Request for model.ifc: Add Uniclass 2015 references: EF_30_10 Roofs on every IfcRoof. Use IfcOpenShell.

First a look at what the model holds.

```python
import ifcopenshell

model = ifcopenshell.open("model.ifc")
print(model.schema)
print("classifications:", [c.Name for c in model.by_type("IfcClassification")])
for ifc_class in ("IfcDoor", "IfcRoof", "IfcStair", "IfcWall", "IfcWindow"):
    print(ifc_class, len(model.by_type(ifc_class)))
```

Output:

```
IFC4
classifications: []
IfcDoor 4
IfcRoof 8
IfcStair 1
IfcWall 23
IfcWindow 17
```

```python
import ifcopenshell
import ifcopenshell.api.classification

model = ifcopenshell.open("model.ifc")

system = ifcopenshell.api.classification.add_classification(model, classification="Uniclass 2015")

codes = {
    "IfcRoof": ("EF_30_10", "Roofs"),
}
for ifc_class, (code, name) in codes.items():
    products = model.by_type(ifc_class)
    ifcopenshell.api.classification.add_reference(
        model, products=products, classification=system, identification=code, name=name
    )
    print(code, len(products))

model.write("model_rev.ifc")
```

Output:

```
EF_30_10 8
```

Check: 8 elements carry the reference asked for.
